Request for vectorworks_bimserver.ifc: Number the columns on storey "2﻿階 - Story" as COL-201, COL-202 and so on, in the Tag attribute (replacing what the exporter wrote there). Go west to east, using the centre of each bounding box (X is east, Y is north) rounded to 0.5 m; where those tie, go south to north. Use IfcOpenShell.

First a look at what the model holds.

```python
import ifcopenshell
import ifcopenshell.util.element
import ifcopenshell.util.placement

model = ifcopenshell.open("vectorworks_bimserver.ifc")
print(model.schema)
storey = next(s for s in model.by_type("IfcBuildingStorey") if s.Name == '2\ufeff階 - Story')
columns = [e for e in ifcopenshell.util.element.get_decomposition(storey) if e.is_a("IfcColumn")]
for e in sorted(columns, key=lambda e: e.id()):
    origin = ifcopenshell.util.placement.get_local_placement(e.ObjectPlacement)[:3, 3]
    print(e.id(), e.Tag, e.Name, origin.round(2) + 0.0, sep=" | ")
```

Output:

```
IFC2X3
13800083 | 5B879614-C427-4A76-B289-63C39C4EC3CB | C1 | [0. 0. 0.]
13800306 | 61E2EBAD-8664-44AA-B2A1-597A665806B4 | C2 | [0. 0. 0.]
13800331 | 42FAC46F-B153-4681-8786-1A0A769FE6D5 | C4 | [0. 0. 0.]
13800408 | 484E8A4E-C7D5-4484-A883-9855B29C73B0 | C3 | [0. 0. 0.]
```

```python
import ifcopenshell
import ifcopenshell.geom
import ifcopenshell.util.element
import ifcopenshell.util.shape

model = ifcopenshell.open("vectorworks_bimserver.ifc")
settings = ifcopenshell.geom.settings()
settings.set("use-world-coords", True)


def centre(element):
    shape = ifcopenshell.geom.create_shape(settings, element)
    return ifcopenshell.util.shape.get_bbox_centroid(shape.geometry)


storey = next(s for s in model.by_type("IfcBuildingStorey") if s.Name == '2\ufeff階 - Story')
columns = [e for e in ifcopenshell.util.element.get_decomposition(storey) if e.is_a("IfcColumn")]

# Insertion points can sit at a corner or the storey origin, so sort by the geometry (in metres).
centres = {e: centre(e) for e in columns}
columns.sort(key=lambda e: (round(centres[e][0] / 0.5), centres[e][1]))

for i, e in enumerate(columns, start=1):
    number = f"COL-2{i:02d}"
    e.Tag = number
    print(e.id(), number)

model.write("vectorworks_bimserver_edited.ifc")
```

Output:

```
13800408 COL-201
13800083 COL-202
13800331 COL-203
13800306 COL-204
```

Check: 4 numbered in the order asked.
